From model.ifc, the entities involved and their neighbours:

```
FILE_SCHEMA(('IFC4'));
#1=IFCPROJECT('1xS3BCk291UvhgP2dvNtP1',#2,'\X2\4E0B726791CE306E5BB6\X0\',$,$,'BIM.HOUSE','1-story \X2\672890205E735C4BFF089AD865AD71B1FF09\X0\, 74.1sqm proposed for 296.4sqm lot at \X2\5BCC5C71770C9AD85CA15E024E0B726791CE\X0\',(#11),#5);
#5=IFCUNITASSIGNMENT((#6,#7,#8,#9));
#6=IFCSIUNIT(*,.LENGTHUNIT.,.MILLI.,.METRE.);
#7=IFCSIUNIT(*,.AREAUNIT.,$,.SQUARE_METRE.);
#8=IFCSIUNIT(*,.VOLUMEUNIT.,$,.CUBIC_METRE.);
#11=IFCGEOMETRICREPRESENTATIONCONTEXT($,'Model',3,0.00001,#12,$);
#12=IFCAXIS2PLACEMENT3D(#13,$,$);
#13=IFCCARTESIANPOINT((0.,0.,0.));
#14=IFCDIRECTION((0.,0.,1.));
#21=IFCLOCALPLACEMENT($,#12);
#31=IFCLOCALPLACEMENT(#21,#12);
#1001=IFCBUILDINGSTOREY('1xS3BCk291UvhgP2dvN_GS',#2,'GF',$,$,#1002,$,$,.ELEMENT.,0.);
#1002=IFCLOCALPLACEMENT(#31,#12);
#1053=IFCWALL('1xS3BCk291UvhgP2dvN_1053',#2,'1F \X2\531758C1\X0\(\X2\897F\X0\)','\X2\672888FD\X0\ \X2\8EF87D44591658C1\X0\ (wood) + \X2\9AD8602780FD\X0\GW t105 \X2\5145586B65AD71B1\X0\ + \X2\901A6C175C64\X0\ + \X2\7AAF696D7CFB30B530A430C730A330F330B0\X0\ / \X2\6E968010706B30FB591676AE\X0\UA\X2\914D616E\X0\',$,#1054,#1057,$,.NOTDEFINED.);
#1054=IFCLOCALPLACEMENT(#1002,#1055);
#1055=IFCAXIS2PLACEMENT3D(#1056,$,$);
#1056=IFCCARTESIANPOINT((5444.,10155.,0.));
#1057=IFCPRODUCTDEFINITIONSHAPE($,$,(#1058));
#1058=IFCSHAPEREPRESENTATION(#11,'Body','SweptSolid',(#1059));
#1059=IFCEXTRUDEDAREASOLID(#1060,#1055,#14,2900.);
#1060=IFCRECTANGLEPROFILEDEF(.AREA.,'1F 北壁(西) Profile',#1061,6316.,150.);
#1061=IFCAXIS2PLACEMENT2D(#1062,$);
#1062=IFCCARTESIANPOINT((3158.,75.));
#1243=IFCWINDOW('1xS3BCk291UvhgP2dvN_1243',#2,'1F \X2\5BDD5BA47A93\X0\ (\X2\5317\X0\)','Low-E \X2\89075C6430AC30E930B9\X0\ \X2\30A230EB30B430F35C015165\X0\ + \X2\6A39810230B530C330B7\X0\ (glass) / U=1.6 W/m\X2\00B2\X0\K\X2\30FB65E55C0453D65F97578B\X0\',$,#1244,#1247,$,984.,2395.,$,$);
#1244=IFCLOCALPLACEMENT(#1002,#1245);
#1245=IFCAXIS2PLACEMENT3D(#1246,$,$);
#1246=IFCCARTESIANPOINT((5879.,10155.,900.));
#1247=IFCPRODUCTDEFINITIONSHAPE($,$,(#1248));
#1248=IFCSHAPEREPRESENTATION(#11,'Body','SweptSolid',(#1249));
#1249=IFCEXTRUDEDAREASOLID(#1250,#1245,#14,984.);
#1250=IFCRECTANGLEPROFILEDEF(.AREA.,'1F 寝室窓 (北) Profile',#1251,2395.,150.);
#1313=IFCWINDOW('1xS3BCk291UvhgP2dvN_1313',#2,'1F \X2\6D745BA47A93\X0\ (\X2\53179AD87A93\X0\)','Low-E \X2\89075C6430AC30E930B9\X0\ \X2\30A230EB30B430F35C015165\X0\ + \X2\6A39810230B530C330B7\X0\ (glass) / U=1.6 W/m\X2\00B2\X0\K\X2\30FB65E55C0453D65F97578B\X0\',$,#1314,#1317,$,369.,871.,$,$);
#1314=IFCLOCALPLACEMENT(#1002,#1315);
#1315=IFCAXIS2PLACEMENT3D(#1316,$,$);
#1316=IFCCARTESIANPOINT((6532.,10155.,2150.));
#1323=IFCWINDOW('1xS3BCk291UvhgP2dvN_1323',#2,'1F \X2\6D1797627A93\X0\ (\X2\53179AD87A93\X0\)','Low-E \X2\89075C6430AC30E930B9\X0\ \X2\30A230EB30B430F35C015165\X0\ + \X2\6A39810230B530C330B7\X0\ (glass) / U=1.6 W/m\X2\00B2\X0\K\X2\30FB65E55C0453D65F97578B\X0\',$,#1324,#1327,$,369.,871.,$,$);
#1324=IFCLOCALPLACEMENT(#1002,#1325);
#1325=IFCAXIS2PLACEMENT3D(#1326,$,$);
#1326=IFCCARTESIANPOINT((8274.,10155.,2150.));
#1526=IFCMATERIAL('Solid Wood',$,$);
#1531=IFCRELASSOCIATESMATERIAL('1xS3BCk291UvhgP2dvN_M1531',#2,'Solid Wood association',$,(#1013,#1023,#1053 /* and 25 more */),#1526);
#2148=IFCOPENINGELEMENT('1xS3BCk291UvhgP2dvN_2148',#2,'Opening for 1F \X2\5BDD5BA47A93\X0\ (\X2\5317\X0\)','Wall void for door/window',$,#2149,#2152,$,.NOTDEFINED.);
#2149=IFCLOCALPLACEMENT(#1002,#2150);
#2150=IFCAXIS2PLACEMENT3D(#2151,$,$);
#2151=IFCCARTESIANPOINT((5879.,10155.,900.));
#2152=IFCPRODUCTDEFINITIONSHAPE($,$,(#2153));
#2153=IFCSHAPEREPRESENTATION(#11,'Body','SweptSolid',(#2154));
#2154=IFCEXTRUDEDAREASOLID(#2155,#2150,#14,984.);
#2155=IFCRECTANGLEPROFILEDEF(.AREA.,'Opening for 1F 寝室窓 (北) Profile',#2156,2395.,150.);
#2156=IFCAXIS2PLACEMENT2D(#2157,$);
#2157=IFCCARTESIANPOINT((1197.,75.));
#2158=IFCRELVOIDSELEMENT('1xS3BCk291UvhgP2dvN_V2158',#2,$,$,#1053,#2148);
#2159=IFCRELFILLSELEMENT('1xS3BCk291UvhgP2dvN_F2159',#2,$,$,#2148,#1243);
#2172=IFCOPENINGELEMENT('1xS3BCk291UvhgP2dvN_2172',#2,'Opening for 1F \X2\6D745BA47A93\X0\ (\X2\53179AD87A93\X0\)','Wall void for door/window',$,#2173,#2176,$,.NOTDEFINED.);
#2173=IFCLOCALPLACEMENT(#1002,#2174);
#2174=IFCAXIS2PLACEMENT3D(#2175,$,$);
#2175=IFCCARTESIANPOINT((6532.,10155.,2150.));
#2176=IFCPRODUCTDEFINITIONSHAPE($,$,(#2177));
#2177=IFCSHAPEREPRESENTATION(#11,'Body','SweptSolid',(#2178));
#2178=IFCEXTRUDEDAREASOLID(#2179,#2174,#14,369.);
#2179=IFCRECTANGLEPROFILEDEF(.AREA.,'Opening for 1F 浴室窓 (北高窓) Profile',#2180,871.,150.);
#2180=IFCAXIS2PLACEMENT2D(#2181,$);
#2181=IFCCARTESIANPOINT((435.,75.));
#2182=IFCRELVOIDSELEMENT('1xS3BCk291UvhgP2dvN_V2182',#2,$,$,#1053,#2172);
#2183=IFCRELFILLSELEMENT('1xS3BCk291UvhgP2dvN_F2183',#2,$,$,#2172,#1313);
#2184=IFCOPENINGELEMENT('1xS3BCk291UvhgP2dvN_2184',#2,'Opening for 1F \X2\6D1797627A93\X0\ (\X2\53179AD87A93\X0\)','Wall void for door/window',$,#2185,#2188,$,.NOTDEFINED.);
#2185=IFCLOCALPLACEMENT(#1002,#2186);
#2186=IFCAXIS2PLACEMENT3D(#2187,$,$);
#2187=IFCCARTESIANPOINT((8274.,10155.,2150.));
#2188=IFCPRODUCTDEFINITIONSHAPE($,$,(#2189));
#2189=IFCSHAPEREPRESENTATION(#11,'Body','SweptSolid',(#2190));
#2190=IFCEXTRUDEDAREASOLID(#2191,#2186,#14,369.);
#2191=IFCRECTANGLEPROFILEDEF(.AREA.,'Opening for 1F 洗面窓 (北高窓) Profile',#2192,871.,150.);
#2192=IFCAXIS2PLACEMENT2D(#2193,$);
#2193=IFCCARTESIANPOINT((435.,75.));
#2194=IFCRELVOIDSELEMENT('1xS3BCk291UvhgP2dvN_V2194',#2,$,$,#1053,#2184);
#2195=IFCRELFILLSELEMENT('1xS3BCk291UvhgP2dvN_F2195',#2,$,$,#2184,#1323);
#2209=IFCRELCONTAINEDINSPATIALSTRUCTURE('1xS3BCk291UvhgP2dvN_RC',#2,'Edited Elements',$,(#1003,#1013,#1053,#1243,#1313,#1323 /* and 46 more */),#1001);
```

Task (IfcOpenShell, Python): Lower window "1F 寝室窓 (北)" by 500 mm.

```python
import numpy as np
import ifcopenshell
import ifcopenshell.api.geometry
import ifcopenshell.util.placement
import ifcopenshell.util.unit

model = ifcopenshell.open("model.ifc")
unit_scale = ifcopenshell.util.unit.calculate_unit_scale(model)

window = model.by_guid("1xS3BCk291UvhgP2dvN_1243")
opening = window.FillsVoids[0].RelatingOpeningElement
dz = -500.0

shift = np.array([0.0, 0.0, dz])
# The window is not placed relative to its opening, so move both.
for product in (opening, window):
    matrix = ifcopenshell.util.placement.get_local_placement(product.ObjectPlacement)
    matrix[:3, 3] += shift
    ifcopenshell.api.geometry.edit_object_placement(model, product=product, matrix=matrix, is_si=False)

print(f"moved by {dz * unit_scale:+.3f} m")

model.write("model_edited.ifc")
```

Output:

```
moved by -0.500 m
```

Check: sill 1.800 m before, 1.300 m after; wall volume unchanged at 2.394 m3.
